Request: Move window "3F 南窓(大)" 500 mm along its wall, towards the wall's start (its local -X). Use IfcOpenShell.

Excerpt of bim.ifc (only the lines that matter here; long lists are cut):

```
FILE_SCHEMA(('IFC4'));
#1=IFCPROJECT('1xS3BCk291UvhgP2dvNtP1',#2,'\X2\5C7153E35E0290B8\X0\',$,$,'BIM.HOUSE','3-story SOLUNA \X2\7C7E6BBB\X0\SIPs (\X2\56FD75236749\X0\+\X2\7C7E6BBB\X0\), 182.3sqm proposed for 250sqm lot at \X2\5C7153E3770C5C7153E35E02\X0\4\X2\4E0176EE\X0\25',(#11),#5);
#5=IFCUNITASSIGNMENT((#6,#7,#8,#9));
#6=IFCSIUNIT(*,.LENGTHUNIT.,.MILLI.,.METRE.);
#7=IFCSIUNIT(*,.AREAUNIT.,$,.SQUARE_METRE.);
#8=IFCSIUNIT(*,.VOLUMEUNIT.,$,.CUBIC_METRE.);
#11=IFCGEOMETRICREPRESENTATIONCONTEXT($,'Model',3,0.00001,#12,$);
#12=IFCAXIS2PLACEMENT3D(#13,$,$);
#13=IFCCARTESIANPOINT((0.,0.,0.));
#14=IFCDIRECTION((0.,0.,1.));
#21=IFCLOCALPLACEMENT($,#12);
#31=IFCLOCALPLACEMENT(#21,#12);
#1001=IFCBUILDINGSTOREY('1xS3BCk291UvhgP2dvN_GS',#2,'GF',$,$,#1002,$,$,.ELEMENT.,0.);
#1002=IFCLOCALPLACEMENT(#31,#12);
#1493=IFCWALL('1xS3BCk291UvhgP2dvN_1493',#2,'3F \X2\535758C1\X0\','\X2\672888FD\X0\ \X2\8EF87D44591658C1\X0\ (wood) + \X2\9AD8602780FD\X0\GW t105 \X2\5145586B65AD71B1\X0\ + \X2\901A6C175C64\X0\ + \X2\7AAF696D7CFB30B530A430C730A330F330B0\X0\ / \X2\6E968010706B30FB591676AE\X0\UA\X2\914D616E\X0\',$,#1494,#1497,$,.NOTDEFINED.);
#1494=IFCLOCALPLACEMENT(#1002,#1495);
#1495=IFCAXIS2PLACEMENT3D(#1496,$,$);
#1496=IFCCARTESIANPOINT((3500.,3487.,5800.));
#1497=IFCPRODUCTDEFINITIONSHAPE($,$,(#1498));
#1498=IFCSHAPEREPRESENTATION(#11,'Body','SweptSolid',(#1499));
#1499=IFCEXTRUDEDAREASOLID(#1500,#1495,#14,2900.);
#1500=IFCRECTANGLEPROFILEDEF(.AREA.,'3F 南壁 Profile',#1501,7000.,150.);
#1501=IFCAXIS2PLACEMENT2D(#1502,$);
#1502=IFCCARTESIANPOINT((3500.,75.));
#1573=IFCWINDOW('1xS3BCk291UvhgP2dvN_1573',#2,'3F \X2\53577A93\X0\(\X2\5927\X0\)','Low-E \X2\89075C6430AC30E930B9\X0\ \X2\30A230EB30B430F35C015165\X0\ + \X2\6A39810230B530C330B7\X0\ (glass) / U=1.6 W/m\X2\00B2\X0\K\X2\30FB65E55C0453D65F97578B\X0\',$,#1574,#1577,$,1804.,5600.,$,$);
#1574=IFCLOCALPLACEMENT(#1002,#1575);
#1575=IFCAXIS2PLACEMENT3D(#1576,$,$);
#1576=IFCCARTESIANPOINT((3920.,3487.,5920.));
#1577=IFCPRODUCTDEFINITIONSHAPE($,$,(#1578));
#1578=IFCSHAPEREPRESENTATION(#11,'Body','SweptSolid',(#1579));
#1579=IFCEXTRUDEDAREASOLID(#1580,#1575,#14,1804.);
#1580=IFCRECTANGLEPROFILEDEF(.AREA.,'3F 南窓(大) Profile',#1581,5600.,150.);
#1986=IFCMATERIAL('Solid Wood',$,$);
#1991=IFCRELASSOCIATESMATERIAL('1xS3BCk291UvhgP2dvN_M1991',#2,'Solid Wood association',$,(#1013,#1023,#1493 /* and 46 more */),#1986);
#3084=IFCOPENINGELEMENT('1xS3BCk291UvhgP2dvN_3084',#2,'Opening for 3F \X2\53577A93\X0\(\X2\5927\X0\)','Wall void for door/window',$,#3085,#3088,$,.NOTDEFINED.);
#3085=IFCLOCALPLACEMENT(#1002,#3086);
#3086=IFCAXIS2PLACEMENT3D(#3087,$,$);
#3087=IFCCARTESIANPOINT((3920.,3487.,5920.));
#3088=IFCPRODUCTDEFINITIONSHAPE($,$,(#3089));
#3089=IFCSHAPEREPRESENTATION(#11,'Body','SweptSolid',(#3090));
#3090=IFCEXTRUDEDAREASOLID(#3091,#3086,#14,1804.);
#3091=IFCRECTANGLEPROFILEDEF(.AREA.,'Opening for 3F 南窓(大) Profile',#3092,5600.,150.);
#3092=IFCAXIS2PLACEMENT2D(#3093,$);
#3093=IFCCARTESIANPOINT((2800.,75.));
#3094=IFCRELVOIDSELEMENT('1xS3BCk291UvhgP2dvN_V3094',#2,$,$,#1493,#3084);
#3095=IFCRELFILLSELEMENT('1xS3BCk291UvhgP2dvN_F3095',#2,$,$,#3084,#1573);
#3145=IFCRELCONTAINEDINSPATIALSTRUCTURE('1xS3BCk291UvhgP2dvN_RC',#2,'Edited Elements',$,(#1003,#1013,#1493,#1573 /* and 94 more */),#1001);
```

```python
import ifcopenshell
import ifcopenshell.api.geometry
import ifcopenshell.util.placement
import ifcopenshell.util.unit

model = ifcopenshell.open("bim.ifc")
unit_scale = ifcopenshell.util.unit.calculate_unit_scale(model)

window = model.by_guid("1xS3BCk291UvhgP2dvN_1573")
opening = window.FillsVoids[0].RelatingOpeningElement
wall = opening.VoidsElements[0].RelatingBuildingElement

wall_matrix = ifcopenshell.util.placement.get_local_placement(wall.ObjectPlacement)
shift = wall_matrix[:3, 0] * -0.5 / unit_scale
before = ifcopenshell.util.placement.get_local_placement(window.ObjectPlacement)[:3, 3].copy()

# The window is not placed relative to its opening, so move both.
for product in (opening, window):
    matrix = ifcopenshell.util.placement.get_local_placement(product.ObjectPlacement)
    matrix[:3, 3] += shift
    ifcopenshell.api.geometry.edit_object_placement(model, product=product, matrix=matrix, is_si=False)

after = ifcopenshell.util.placement.get_local_placement(window.ObjectPlacement)[:3, 3]
print("window moved by", (after - before).round(3) + 0.0)

model.write("bim_edited.ifc")
```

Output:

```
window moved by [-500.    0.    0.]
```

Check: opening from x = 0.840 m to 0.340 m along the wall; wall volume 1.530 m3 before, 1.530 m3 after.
